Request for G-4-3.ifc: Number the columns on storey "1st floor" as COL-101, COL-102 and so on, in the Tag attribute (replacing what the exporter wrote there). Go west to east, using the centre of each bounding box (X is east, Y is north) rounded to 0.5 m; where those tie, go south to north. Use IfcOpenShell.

First a look at what the model holds.

```python
import ifcopenshell
import ifcopenshell.util.element
import ifcopenshell.util.placement

model = ifcopenshell.open("G-4-3.ifc")
print(model.schema)
storey = next(s for s in model.by_type("IfcBuildingStorey") if s.Name == "1st floor")
columns = [e for e in ifcopenshell.util.element.get_decomposition(storey) if e.is_a("IfcColumn")]
for e in sorted(columns, key=lambda e: e.id()):
    origin = ifcopenshell.util.placement.get_local_placement(e.ObjectPlacement)[:3, 3]
    print(e.id(), e.Tag, e.Name, origin.round(2) + 0.0, sep=" | ")
```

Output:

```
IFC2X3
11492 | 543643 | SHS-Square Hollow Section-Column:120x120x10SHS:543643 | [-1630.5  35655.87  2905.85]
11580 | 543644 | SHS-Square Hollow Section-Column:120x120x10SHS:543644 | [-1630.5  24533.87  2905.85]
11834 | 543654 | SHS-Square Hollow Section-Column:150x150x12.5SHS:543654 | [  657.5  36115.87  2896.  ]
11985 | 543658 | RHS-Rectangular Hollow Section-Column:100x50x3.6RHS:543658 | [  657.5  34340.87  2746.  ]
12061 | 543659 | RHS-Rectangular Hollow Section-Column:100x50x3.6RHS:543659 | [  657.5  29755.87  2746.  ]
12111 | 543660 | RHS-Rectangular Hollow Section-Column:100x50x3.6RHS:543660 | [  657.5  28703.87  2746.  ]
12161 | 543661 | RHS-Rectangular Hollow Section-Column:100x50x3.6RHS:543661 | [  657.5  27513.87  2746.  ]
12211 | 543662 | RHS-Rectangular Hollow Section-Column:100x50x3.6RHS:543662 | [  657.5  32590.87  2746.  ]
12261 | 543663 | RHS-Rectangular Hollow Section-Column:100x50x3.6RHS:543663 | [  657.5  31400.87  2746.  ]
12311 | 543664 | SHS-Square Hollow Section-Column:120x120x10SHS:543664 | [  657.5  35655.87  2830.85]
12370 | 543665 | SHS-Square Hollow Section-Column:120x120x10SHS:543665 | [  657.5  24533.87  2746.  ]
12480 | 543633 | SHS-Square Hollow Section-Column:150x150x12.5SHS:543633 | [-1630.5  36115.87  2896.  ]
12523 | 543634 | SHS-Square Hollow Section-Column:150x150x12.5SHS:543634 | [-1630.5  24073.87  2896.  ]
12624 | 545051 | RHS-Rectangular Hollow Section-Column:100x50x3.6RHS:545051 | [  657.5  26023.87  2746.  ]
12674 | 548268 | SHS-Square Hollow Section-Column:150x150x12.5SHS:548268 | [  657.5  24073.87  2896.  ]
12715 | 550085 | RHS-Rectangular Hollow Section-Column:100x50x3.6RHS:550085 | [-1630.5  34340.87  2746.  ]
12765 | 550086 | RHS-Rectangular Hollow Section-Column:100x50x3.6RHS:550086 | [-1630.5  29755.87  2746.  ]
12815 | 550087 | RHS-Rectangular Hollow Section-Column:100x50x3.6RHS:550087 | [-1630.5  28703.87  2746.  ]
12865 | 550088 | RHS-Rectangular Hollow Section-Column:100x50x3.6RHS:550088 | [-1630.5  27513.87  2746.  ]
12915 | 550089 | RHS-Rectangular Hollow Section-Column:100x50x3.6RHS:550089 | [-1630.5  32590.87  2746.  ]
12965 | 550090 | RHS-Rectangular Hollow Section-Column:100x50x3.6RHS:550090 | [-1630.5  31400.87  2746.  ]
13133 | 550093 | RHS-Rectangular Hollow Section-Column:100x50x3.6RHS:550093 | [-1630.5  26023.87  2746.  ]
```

```python
import ifcopenshell
import ifcopenshell.geom
import ifcopenshell.util.element
import ifcopenshell.util.shape

model = ifcopenshell.open("G-4-3.ifc")
settings = ifcopenshell.geom.settings()
settings.set("use-world-coords", True)


def centre(element):
    shape = ifcopenshell.geom.create_shape(settings, element)
    return ifcopenshell.util.shape.get_bbox_centroid(shape.geometry)


storey = next(s for s in model.by_type("IfcBuildingStorey") if s.Name == "1st floor")
columns = [e for e in ifcopenshell.util.element.get_decomposition(storey) if e.is_a("IfcColumn")]

# Insertion points can sit at a corner or the storey origin, so sort by the geometry (in metres).
centres = {e: centre(e) for e in columns}
columns.sort(key=lambda e: (round(centres[e][0] / 0.5), centres[e][1]))

for i, e in enumerate(columns, start=1):
    number = f"COL-1{i:02d}"
    e.Tag = number
    print(e.id(), number)

model.write("G-4-3_v2.ifc")
```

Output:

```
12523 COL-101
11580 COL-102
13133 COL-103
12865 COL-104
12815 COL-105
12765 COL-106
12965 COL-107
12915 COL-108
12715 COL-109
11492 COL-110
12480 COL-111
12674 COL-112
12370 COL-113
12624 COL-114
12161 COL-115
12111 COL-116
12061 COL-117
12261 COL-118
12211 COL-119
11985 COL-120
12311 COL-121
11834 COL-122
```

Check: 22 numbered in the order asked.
